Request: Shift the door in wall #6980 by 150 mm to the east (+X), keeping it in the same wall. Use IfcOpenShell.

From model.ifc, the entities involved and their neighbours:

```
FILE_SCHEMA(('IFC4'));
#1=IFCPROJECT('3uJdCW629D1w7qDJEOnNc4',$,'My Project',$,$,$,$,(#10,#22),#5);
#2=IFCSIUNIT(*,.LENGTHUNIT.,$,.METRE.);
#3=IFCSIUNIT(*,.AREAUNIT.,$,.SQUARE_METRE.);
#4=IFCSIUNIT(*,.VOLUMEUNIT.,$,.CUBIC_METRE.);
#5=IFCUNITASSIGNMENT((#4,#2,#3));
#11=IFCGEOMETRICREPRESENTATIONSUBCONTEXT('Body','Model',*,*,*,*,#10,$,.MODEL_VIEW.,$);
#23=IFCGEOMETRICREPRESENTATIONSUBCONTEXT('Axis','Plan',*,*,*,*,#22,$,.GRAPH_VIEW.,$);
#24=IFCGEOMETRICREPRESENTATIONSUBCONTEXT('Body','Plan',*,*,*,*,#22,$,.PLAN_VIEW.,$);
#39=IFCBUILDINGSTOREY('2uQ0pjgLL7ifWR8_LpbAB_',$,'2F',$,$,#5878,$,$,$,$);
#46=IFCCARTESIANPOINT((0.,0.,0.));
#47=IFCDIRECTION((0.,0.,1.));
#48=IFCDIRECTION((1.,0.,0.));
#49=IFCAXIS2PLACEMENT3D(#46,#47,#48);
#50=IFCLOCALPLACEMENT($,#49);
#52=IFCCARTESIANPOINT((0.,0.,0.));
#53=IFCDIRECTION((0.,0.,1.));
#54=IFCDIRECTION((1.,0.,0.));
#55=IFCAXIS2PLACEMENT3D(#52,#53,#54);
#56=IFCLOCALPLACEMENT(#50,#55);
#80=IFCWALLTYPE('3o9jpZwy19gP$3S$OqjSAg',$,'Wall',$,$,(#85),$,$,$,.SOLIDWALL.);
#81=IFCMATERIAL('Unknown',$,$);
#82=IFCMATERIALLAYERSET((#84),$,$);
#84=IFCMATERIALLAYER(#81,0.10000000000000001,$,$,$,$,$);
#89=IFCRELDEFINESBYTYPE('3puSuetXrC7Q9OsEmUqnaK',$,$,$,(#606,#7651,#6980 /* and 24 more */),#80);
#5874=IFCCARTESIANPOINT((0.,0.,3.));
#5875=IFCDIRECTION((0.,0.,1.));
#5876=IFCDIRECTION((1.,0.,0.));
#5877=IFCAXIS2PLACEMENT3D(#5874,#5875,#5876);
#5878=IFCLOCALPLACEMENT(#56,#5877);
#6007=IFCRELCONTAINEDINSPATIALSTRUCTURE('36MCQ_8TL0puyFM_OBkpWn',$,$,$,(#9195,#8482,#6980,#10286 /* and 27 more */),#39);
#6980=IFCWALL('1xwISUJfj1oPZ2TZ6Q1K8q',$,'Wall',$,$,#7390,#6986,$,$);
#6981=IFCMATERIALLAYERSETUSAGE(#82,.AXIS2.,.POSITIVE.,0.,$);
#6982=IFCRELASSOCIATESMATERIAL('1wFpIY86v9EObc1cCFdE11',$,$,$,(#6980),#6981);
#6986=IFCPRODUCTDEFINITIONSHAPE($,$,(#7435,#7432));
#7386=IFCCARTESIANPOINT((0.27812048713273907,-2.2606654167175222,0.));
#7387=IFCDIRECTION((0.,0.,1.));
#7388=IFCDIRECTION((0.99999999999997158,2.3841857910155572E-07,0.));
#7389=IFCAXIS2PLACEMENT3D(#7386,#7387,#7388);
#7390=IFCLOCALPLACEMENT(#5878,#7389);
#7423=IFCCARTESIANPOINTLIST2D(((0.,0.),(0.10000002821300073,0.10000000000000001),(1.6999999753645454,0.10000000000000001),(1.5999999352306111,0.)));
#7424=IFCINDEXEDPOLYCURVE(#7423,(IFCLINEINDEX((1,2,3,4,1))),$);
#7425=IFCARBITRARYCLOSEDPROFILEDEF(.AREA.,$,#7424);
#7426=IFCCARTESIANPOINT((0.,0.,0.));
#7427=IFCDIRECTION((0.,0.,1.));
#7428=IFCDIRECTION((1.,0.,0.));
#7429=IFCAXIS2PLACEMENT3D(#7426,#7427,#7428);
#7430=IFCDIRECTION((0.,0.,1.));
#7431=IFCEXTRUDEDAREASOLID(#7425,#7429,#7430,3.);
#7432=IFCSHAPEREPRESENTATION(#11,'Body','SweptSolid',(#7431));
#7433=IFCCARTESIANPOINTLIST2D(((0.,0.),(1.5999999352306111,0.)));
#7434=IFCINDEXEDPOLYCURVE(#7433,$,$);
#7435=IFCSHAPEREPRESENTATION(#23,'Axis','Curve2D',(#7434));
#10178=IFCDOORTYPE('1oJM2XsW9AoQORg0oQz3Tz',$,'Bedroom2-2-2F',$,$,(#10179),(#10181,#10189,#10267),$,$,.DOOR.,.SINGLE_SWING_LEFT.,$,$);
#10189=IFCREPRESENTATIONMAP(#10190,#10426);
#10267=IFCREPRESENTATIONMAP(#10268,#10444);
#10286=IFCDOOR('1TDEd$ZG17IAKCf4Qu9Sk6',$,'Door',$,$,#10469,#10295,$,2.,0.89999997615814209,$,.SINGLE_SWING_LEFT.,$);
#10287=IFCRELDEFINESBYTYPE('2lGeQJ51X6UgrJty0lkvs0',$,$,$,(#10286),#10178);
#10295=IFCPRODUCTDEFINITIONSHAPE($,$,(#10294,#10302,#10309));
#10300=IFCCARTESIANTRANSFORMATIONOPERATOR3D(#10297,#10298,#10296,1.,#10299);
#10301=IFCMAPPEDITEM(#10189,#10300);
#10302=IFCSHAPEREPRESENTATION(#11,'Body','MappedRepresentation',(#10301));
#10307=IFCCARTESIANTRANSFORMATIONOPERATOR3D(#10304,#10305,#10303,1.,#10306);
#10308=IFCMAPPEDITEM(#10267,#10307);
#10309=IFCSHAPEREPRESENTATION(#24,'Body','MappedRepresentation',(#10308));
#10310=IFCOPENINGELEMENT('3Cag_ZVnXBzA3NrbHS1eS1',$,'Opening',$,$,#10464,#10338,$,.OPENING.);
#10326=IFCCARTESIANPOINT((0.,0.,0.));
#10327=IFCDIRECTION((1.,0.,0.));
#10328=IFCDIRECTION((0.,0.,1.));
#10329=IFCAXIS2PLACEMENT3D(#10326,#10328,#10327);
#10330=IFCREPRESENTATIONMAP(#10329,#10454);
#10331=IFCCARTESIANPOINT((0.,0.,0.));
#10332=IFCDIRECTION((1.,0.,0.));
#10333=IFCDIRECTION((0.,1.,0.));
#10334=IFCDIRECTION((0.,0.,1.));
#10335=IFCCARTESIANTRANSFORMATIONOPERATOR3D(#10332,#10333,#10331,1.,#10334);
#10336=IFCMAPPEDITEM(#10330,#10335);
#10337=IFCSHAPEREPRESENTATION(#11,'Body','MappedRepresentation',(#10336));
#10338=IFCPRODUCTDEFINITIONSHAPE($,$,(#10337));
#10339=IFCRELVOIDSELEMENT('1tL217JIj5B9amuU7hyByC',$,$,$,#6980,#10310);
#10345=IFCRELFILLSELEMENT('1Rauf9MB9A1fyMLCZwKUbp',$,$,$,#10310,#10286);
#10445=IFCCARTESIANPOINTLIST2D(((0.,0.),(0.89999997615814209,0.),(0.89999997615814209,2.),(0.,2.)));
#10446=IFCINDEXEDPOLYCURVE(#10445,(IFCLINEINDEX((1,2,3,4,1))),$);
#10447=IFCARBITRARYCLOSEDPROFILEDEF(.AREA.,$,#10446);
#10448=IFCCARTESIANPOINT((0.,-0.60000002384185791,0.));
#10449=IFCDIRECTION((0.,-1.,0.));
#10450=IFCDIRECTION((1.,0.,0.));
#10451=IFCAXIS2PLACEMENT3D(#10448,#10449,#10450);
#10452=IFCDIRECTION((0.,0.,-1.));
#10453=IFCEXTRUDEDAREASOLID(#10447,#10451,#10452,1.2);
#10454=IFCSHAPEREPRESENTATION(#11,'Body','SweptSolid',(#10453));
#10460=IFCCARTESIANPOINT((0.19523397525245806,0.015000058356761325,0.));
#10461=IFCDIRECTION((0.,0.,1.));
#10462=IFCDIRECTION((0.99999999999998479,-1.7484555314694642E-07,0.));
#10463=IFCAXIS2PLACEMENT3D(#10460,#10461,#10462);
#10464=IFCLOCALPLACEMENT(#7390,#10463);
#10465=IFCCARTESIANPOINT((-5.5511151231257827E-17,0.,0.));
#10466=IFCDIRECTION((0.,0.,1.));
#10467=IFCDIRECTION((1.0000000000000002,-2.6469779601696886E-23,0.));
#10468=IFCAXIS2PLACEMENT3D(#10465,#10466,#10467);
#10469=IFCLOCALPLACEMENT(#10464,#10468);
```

```python
import ifcopenshell
import ifcopenshell.api.geometry
import ifcopenshell.util.placement
import ifcopenshell.util.unit

model = ifcopenshell.open("model.ifc")
unit_scale = ifcopenshell.util.unit.calculate_unit_scale(model)

door = model.by_guid("1TDEd$ZG17IAKCf4Qu9Sk6")
opening = door.FillsVoids[0].RelatingOpeningElement
wall = opening.VoidsElements[0].RelatingBuildingElement

wall_matrix = ifcopenshell.util.placement.get_local_placement(wall.ObjectPlacement)
shift = wall_matrix[:3, 0] * 0.15 / unit_scale
before = ifcopenshell.util.placement.get_local_placement(door.ObjectPlacement)[:3, 3].copy()

# The door is placed relative to its opening, so it follows when the opening moves.
matrix = ifcopenshell.util.placement.get_local_placement(opening.ObjectPlacement)
matrix[:3, 3] += shift
ifcopenshell.api.geometry.edit_object_placement(
    model, product=opening, matrix=matrix, is_si=False, should_transform_children=True
)

after = ifcopenshell.util.placement.get_local_placement(door.ObjectPlacement)[:3, 3]
print("door moved by", (after - before).round(3) + 0.0)

model.write("model_rev.ifc")
```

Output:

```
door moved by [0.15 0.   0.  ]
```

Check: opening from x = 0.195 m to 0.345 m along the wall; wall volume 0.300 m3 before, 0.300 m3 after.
